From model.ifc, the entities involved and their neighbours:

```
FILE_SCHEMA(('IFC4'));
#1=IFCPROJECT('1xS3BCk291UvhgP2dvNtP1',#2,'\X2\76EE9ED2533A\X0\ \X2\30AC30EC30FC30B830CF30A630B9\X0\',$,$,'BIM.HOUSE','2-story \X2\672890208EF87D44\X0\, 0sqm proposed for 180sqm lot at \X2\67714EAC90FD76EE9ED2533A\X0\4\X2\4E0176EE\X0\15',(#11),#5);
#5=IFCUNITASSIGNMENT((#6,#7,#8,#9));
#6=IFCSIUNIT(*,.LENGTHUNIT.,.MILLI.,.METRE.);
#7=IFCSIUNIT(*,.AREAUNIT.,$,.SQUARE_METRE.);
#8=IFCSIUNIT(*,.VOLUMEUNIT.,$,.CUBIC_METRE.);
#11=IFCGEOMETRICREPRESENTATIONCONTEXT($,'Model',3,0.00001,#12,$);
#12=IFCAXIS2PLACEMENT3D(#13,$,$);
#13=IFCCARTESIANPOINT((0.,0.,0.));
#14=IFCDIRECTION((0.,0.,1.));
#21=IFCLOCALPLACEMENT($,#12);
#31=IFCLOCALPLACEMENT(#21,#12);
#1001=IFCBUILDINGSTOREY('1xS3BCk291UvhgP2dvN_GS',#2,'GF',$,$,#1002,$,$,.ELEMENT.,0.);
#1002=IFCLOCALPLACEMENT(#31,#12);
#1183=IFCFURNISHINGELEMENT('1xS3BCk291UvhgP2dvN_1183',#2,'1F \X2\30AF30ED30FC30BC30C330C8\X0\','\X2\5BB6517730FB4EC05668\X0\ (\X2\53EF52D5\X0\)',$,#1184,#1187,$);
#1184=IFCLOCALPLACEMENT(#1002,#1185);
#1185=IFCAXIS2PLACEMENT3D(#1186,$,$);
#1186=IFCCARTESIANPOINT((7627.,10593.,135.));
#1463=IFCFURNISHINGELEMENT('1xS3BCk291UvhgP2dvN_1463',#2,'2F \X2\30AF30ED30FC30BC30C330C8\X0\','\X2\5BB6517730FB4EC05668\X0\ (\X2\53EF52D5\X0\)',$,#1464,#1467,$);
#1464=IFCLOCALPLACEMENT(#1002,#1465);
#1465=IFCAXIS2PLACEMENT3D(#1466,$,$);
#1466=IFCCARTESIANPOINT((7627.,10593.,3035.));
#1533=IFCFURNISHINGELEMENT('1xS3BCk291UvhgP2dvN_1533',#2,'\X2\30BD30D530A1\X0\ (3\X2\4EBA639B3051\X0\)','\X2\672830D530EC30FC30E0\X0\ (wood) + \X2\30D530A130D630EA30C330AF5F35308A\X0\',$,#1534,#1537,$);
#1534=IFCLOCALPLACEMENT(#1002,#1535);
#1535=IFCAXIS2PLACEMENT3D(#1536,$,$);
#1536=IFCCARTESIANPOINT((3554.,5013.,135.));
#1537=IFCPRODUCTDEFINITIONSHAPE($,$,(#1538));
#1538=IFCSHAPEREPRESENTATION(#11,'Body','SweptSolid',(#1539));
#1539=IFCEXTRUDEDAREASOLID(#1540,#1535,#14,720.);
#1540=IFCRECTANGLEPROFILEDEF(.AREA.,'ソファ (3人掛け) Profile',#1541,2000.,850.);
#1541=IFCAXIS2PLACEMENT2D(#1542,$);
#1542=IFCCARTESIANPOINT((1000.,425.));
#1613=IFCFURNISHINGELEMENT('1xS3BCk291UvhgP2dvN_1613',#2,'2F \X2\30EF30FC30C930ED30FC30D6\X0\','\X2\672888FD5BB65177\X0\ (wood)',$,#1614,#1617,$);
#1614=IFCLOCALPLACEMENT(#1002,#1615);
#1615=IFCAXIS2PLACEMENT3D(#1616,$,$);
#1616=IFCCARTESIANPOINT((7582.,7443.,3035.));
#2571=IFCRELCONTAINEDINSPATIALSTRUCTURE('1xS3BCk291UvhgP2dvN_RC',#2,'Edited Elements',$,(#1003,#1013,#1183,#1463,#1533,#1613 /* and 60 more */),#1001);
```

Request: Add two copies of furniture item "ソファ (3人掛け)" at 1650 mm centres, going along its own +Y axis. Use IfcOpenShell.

```python
import ifcopenshell
import ifcopenshell.api.geometry
import ifcopenshell.api.root
import ifcopenshell.util.element
import ifcopenshell.util.placement

model = ifcopenshell.open("model.ifc")


def reuse_history(source, copy):
    """copy_class also copies each property set's owner history, people and application; keep the originals."""
    for rel in copy.IsDefinedBy:
        if rel.is_a("IfcRelDefinesByProperties") and (history := rel.RelatingPropertyDefinition.OwnerHistory):
            rel.RelatingPropertyDefinition.OwnerHistory = source.OwnerHistory
            ifcopenshell.util.element.remove_deep2(model, history)


source = model.by_id(1533)
base = ifcopenshell.util.placement.get_local_placement(source.ObjectPlacement)
step = base[:3, 1] * 1650.0

for i in range(1, 3):
    copy = ifcopenshell.api.root.copy_class(model, product=source)
    copy.Representation = ifcopenshell.util.element.copy_deep(
        model, source.Representation, exclude=["IfcGeometricRepresentationContext", "IfcRepresentationMap"]
    )
    reuse_history(source, copy)
    matrix = base.copy()
    matrix[:3, 3] += i * step
    print("added at", matrix[:3, 3].round(3) + 0.0)
    ifcopenshell.api.geometry.edit_object_placement(model, product=copy, matrix=matrix, is_si=False)

model.write("model_updated.ifc")
```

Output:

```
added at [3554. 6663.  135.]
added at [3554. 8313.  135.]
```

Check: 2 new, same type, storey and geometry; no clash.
